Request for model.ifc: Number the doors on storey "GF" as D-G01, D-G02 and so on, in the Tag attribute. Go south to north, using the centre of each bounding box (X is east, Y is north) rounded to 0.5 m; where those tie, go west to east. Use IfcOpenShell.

First a look at what the model holds.

```python
import ifcopenshell
import ifcopenshell.util.element
import ifcopenshell.util.placement

model = ifcopenshell.open("model.ifc")
print(model.schema)
storey = next(s for s in model.by_type("IfcBuildingStorey") if s.Name == "GF")
doors = [e for e in ifcopenshell.util.element.get_decomposition(storey) if e.is_a("IfcDoor")]
for e in sorted(doors, key=lambda e: e.id()):
    origin = ifcopenshell.util.placement.get_local_placement(e.ObjectPlacement)[:3, 3]
    print(e.id(), e.Tag, e.Name, origin.round(2) + 0.0, sep=" | ")
```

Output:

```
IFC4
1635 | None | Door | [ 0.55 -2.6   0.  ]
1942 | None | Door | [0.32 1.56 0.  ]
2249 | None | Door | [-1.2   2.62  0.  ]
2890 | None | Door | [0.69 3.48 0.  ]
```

```python
import ifcopenshell
import ifcopenshell.geom
import ifcopenshell.util.element
import ifcopenshell.util.shape

model = ifcopenshell.open("model.ifc")
settings = ifcopenshell.geom.settings()
settings.set("use-world-coords", True)


def centre(element):
    shape = ifcopenshell.geom.create_shape(settings, element)
    return ifcopenshell.util.shape.get_bbox_centroid(shape.geometry)


storey = next(s for s in model.by_type("IfcBuildingStorey") if s.Name == "GF")
doors = [e for e in ifcopenshell.util.element.get_decomposition(storey) if e.is_a("IfcDoor")]

# Insertion points can sit at a corner or the storey origin, so sort by the geometry (in metres).
centres = {e: centre(e) for e in doors}
doors.sort(key=lambda e: (round(centres[e][1] / 0.5), centres[e][0]))

for i, e in enumerate(doors, start=1):
    number = f"D-G{i:02d}"
    e.Tag = number
    print(e.id(), number)

model.write("model_edited.ifc")
```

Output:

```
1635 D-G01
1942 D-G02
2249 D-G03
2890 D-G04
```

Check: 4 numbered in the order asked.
